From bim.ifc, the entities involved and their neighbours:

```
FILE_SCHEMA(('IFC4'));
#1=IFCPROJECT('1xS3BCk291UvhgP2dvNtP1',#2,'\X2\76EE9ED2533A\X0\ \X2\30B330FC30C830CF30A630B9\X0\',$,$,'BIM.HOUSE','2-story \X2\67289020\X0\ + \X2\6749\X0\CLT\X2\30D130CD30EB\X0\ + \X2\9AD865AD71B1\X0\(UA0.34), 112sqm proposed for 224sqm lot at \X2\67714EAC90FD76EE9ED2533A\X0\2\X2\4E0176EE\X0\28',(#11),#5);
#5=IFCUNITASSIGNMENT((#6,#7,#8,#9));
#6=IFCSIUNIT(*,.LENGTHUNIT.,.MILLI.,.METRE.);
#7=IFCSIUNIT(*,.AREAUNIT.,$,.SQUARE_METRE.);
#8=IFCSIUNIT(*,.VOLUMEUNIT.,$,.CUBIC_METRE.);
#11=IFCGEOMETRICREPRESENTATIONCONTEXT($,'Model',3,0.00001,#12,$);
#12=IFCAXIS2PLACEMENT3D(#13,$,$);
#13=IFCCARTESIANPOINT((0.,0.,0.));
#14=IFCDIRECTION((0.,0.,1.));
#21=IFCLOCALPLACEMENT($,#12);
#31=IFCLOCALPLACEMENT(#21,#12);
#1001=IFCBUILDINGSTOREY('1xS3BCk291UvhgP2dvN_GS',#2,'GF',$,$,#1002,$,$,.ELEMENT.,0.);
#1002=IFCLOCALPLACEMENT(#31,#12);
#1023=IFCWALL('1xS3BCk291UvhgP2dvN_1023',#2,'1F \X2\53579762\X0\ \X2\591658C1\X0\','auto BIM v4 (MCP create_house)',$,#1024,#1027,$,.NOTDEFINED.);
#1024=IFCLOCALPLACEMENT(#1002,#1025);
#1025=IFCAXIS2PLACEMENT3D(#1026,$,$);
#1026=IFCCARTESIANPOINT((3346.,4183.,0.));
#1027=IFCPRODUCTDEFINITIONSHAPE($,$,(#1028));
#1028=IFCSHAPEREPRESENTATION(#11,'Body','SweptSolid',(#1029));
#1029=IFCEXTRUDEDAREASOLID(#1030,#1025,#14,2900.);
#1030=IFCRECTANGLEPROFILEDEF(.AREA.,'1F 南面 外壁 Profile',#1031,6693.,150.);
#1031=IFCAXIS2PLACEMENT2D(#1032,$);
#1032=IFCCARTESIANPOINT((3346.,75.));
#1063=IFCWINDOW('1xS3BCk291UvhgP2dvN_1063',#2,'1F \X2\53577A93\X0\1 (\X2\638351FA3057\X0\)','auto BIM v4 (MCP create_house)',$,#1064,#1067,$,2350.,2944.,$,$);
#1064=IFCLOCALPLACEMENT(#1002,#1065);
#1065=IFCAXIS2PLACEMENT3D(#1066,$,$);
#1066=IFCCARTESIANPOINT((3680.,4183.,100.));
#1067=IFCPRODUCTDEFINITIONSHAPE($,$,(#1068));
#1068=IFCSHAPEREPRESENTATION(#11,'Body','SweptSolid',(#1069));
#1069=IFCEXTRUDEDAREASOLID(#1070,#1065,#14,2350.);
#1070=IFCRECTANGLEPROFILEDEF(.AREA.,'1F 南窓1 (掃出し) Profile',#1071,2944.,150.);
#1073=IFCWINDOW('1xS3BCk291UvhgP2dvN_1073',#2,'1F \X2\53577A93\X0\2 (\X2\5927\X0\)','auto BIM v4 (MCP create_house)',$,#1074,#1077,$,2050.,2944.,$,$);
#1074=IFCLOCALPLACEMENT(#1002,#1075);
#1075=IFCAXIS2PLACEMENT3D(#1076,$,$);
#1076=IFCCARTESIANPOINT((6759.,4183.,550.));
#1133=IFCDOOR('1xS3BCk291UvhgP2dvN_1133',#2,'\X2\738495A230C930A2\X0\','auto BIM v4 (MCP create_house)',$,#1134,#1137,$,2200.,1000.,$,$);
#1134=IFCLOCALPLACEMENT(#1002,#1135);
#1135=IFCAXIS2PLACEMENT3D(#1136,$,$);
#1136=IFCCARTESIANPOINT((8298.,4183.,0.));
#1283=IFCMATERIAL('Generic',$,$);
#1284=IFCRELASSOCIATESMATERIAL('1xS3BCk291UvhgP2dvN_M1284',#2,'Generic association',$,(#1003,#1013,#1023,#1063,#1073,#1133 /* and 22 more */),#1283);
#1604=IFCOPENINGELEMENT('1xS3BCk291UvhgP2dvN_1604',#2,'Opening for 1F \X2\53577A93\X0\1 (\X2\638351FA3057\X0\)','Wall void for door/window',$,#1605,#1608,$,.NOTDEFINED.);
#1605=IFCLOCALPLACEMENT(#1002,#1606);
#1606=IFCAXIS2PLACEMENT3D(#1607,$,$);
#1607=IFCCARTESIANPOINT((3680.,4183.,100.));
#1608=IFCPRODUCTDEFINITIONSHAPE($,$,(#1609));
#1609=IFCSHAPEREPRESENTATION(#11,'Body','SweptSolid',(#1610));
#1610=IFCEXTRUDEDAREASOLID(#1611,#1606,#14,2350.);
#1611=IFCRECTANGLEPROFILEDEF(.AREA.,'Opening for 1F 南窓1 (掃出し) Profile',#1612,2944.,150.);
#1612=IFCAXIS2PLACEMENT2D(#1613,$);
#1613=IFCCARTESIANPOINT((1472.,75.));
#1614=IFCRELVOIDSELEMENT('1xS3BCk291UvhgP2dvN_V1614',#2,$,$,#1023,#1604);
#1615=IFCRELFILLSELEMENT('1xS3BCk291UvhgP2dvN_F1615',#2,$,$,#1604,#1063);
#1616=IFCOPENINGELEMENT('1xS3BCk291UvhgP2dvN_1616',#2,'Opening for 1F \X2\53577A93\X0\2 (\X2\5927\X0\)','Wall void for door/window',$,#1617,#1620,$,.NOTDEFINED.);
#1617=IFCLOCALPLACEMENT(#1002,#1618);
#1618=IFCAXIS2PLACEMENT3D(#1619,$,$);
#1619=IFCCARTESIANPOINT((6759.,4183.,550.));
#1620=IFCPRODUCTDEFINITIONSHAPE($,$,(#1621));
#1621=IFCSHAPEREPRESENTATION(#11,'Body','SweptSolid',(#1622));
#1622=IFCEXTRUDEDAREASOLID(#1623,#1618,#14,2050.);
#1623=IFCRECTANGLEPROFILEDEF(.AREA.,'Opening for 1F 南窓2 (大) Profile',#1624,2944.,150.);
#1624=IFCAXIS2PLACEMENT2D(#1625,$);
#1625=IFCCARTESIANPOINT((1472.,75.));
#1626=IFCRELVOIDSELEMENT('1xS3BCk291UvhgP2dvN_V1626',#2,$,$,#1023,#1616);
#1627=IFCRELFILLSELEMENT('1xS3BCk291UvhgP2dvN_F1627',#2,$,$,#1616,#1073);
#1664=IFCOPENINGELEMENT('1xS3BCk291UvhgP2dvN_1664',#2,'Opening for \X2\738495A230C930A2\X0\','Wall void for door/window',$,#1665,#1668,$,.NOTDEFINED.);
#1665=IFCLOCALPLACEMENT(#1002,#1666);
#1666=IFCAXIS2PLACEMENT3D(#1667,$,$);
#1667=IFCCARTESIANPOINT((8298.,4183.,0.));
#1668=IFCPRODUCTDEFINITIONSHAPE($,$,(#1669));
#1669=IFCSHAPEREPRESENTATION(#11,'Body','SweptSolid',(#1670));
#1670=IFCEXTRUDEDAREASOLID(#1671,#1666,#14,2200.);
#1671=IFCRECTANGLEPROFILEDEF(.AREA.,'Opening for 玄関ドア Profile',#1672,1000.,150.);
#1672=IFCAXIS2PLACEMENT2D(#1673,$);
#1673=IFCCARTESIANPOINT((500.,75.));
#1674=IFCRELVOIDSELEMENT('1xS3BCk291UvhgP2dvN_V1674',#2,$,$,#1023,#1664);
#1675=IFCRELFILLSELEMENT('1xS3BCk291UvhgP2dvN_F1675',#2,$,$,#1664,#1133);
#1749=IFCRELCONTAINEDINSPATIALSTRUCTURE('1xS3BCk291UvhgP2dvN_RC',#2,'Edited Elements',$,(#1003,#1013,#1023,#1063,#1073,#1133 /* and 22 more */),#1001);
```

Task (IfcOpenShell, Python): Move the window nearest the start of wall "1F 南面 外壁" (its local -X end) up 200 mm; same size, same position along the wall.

```python
import numpy as np
import ifcopenshell
import ifcopenshell.api.geometry
import ifcopenshell.util.placement
import ifcopenshell.util.unit

model = ifcopenshell.open("bim.ifc")
unit_scale = ifcopenshell.util.unit.calculate_unit_scale(model)

window = model.by_guid("1xS3BCk291UvhgP2dvN_1063")
opening = window.FillsVoids[0].RelatingOpeningElement
dz = 0.2 / unit_scale

shift = np.array([0.0, 0.0, dz])
# The window is not placed relative to its opening, so move both.
for product in (opening, window):
    matrix = ifcopenshell.util.placement.get_local_placement(product.ObjectPlacement)
    matrix[:3, 3] += shift
    ifcopenshell.api.geometry.edit_object_placement(model, product=product, matrix=matrix, is_si=False)

print(f"moved by {dz * unit_scale:+.3f} m")

model.write("bim_edited.ifc")
```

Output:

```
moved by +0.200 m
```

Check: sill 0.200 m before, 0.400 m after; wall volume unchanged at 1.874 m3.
